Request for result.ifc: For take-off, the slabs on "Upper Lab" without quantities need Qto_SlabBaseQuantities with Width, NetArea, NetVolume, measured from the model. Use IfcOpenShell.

First a look at what the model holds.

```python
import ifcopenshell
import ifcopenshell.util.element
import ifcopenshell.util.unit

model = ifcopenshell.open("result.ifc")
print(model.schema)
for unit_type in ("LENGTHUNIT", "AREAUNIT", "VOLUMEUNIT"):
    print(unit_type, ifcopenshell.util.unit.calculate_unit_scale(model, unit_type))
storey = next(s for s in model.by_type("IfcBuildingStorey") if s.Name == "Upper Lab")
slabs = [e for e in ifcopenshell.util.element.get_decomposition(storey) if e.is_a("IfcSlab")]
for e in sorted(slabs, key=lambda e: e.id()):
    print(e.id(), e.is_a(), e.Name, list(ifcopenshell.util.element.get_psets(e, qtos_only=True)), sep=" | ")
```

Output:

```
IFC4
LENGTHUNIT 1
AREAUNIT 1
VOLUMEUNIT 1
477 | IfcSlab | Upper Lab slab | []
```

```python
import ifcopenshell
import ifcopenshell.api.pset
import ifcopenshell.geom
import ifcopenshell.util.element
import ifcopenshell.util.shape
import ifcopenshell.util.unit

model = ifcopenshell.open("result.ifc")
unit_scale = ifcopenshell.util.unit.calculate_unit_scale(model)
area_scale = ifcopenshell.util.unit.calculate_unit_scale(model, "AREAUNIT")
volume_scale = ifcopenshell.util.unit.calculate_unit_scale(model, "VOLUMEUNIT")
settings = ifcopenshell.geom.settings()

storey = next(s for s in model.by_type("IfcBuildingStorey") if s.Name == "Upper Lab")
slabs = [e for e in ifcopenshell.util.element.get_decomposition(storey) if e.is_a("IfcSlab")]

for e in sorted(slabs, key=lambda e: e.id()):
    if ifcopenshell.util.element.get_psets(e, qtos_only=True, should_inherit=False):
        continue
    # Geometry comes back in metres, in the element's own axes.
    shape = ifcopenshell.geom.create_shape(settings, e)
    values = {
        "Width": ifcopenshell.util.shape.get_z(shape.geometry) / unit_scale,
        "NetArea": ifcopenshell.util.shape.get_footprint_area(shape.geometry) / area_scale,
        "NetVolume": ifcopenshell.util.shape.get_volume(shape.geometry) / volume_scale,
    }
    qto = ifcopenshell.api.pset.add_qto(model, product=e, name="Qto_SlabBaseQuantities")
    ifcopenshell.api.pset.edit_qto(model, qto=qto, properties=values)
    print(e.id(), {k: round(v, 3) for k, v in values.items()})

model.write("result_v2.ifc")
```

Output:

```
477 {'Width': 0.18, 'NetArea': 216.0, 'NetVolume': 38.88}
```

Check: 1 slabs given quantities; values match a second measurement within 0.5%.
